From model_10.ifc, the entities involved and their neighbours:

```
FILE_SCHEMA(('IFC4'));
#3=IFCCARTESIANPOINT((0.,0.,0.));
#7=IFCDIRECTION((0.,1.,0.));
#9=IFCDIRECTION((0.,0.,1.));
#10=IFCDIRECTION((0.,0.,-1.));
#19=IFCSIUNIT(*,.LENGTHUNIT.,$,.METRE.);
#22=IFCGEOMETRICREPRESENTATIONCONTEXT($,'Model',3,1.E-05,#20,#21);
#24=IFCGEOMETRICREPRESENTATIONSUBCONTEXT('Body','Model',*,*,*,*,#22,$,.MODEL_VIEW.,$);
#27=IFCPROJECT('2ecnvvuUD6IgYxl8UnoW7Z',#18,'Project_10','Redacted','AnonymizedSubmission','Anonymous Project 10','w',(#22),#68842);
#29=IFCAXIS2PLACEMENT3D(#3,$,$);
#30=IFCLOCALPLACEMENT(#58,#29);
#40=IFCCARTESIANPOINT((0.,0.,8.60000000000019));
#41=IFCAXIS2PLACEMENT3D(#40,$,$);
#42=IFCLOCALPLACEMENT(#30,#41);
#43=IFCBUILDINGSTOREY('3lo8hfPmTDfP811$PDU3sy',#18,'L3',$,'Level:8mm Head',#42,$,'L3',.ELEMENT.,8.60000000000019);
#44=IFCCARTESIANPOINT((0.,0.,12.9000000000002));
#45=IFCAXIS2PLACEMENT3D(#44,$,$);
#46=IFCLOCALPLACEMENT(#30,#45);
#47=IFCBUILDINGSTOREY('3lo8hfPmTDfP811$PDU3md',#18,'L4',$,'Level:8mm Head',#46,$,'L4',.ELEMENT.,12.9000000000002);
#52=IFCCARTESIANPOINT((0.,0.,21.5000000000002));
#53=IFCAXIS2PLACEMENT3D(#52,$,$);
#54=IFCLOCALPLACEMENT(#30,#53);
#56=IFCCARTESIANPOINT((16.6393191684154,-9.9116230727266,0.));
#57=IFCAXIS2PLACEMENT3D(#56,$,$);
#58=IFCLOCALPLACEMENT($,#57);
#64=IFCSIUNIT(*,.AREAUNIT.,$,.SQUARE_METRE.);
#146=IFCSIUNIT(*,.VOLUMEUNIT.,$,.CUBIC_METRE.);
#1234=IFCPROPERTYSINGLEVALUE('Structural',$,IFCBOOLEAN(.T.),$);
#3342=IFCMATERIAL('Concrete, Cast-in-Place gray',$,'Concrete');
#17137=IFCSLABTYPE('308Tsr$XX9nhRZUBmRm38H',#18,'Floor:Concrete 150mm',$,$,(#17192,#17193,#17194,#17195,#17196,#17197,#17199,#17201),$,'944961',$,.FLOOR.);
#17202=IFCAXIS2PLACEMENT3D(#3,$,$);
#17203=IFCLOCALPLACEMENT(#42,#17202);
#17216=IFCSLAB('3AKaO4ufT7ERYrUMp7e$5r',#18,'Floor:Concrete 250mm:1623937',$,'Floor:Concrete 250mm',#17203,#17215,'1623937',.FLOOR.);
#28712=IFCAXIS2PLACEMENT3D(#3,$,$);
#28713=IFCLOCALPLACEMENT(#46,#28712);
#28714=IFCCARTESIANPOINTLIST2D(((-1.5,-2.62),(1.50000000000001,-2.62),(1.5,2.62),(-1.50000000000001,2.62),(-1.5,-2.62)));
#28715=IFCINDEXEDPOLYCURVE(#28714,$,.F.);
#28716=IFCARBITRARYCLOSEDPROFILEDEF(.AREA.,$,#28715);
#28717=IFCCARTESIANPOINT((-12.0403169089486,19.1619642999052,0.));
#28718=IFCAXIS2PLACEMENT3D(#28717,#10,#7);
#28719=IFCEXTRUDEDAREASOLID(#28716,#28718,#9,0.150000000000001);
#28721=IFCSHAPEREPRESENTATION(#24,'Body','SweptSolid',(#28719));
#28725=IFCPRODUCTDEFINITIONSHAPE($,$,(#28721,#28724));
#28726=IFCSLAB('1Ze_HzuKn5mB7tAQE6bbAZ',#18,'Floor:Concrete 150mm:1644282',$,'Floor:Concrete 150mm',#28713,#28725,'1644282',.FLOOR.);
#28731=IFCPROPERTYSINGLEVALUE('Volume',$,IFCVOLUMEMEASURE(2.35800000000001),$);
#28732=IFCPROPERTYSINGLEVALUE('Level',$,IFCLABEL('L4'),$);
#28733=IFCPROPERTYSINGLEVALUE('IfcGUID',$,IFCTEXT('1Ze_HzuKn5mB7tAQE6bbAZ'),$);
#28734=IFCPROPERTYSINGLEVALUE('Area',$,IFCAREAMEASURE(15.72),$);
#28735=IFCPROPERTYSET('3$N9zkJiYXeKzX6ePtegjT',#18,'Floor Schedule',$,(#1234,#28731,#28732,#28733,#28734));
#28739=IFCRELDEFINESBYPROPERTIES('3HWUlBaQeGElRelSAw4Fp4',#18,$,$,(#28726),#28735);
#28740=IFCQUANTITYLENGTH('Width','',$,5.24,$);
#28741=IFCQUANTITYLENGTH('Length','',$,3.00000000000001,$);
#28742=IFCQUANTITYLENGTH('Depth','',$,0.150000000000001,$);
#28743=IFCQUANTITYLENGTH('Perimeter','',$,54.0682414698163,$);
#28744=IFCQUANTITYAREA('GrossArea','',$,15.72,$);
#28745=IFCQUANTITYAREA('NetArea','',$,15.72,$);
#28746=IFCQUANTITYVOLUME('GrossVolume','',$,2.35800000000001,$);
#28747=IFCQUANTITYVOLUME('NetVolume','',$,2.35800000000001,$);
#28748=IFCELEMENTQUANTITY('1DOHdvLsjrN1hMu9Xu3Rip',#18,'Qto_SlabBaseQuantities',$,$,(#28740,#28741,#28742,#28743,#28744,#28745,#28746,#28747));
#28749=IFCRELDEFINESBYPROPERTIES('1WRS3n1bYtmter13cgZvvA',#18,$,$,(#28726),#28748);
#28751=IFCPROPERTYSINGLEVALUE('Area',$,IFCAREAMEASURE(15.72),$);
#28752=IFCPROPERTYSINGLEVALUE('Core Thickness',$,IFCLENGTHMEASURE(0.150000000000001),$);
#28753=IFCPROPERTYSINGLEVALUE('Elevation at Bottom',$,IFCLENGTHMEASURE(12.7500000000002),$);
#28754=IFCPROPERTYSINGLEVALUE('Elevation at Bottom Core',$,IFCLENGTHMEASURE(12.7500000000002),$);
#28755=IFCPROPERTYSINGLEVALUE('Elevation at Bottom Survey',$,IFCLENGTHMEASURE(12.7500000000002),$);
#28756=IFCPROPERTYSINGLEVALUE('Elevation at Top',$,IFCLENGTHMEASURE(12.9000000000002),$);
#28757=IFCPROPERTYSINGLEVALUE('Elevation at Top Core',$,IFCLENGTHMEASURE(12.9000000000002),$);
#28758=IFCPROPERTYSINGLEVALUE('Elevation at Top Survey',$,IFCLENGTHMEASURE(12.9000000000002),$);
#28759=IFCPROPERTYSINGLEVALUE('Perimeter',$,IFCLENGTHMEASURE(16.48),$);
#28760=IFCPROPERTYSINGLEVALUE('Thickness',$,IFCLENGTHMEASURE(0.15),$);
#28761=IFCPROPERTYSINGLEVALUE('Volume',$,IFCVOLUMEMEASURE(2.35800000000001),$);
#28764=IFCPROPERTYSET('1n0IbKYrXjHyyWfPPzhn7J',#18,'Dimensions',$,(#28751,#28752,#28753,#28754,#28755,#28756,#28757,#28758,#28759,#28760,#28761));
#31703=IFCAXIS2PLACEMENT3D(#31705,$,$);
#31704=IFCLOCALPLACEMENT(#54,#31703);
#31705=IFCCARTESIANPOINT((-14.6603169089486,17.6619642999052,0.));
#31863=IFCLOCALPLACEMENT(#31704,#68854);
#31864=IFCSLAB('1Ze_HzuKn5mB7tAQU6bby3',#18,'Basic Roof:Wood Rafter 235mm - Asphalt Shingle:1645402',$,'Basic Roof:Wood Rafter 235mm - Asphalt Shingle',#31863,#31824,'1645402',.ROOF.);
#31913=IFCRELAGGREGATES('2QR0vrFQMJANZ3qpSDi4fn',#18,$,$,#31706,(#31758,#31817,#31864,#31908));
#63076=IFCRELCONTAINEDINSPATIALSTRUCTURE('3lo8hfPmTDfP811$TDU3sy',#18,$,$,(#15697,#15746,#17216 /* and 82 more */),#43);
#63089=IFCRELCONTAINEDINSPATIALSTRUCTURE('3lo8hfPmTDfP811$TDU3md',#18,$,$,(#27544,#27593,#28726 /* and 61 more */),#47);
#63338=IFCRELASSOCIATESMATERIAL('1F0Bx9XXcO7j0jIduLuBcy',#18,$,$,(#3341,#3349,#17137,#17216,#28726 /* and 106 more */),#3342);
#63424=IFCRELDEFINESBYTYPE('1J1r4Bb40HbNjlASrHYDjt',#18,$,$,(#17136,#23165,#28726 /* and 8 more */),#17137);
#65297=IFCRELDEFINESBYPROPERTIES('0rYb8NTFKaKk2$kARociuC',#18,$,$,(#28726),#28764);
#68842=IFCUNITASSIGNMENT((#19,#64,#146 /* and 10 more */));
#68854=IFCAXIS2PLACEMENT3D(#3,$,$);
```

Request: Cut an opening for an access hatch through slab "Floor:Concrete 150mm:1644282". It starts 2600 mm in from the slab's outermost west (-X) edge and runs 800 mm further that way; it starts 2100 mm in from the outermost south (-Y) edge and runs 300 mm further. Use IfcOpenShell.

```python
import numpy as np
import ifcopenshell
import ifcopenshell.api.feature
import ifcopenshell.api.geometry
import ifcopenshell.api.pset
import ifcopenshell.api.root
import ifcopenshell.geom
import ifcopenshell.util.element
import ifcopenshell.util.placement
import ifcopenshell.util.representation
import ifcopenshell.util.shape
import ifcopenshell.util.unit

model = ifcopenshell.open("model_10.ifc")
unit_scale = ifcopenshell.util.unit.calculate_unit_scale(model)
area_scale = ifcopenshell.util.unit.calculate_unit_scale(model, "AREAUNIT")
volume_scale = ifcopenshell.util.unit.calculate_unit_scale(model, "VOLUMEUNIT")
settings = ifcopenshell.geom.settings()


def volume(element):
    """Net volume in cubic metres, openings subtracted."""
    shape = ifcopenshell.geom.create_shape(settings, element)
    return ifcopenshell.util.shape.get_volume(shape.geometry)


slab = model.by_id(28726)
before = volume(slab)

# Extent in the slab's own axes, in metres. The edges named are its -X and -Y sides.
slab_shape = ifcopenshell.geom.create_shape(settings, slab)
vertices = ifcopenshell.util.shape.get_vertices(slab_shape.geometry)
x_min, y_min, bottom = vertices.min(axis=0)
top = vertices[:, 2].max()

opening = ifcopenshell.api.root.create_entity(model, ifc_class="IfcOpeningElement", name="Access hatch opening", predefined_type="OPENING")
context = ifcopenshell.util.representation.get_context(model, "Model", "Body", "MODEL_VIEW")
width, depth = 0.8, 0.3
outline = [(0.0, 0.0), (width, 0.0), (width, depth), (0.0, depth), (0.0, 0.0)]
# Overshoot both faces by 50 mm so the cut is clean.
shape = ifcopenshell.api.geometry.add_slab_representation(
    model, context=context, depth=top - bottom + 0.1, polyline=outline
)
ifcopenshell.api.geometry.assign_representation(model, product=opening, representation=shape)

matrix = ifcopenshell.util.placement.get_local_placement(slab.ObjectPlacement)
matrix[:, 3] = matrix @ np.append(np.array([x_min + 2.6, y_min + 2.1, bottom - 0.05]) / unit_scale, 1.0)
ifcopenshell.api.geometry.edit_object_placement(model, product=opening, matrix=matrix, is_si=False)
ifcopenshell.api.feature.add_feature(model, feature=opening, element=slab)

after = volume(slab)

# Update the slab's stored quantities.
pset = model.by_id(ifcopenshell.util.element.get_pset(slab, "Floor Schedule", should_inherit=False)["id"])
ifcopenshell.api.pset.edit_pset(model, pset=pset, properties={
    "Volume": model.create_entity("IfcVolumeMeasure", after / volume_scale),
    "Area": model.create_entity("IfcAreaMeasure", after / (top - bottom) / area_scale),
})
qto = model.by_id(ifcopenshell.util.element.get_pset(slab, "Qto_SlabBaseQuantities", should_inherit=False)["id"])
ifcopenshell.api.pset.edit_qto(model, qto=qto, properties={
    "NetArea": after / (top - bottom) / area_scale,
    "NetVolume": after / volume_scale,
})
pset = model.by_id(ifcopenshell.util.element.get_pset(slab, "Dimensions", should_inherit=False)["id"])
ifcopenshell.api.pset.edit_pset(model, pset=pset, properties={
    "Area": model.create_entity("IfcAreaMeasure", after / (top - bottom) / area_scale),
    "Volume": model.create_entity("IfcVolumeMeasure", after / volume_scale),
})

print(f"slab volume {before:.3f} -> {after:.3f} m3")

model.write("model_10-out.ifc")
```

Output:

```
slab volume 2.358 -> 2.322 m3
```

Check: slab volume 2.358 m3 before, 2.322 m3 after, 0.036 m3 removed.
